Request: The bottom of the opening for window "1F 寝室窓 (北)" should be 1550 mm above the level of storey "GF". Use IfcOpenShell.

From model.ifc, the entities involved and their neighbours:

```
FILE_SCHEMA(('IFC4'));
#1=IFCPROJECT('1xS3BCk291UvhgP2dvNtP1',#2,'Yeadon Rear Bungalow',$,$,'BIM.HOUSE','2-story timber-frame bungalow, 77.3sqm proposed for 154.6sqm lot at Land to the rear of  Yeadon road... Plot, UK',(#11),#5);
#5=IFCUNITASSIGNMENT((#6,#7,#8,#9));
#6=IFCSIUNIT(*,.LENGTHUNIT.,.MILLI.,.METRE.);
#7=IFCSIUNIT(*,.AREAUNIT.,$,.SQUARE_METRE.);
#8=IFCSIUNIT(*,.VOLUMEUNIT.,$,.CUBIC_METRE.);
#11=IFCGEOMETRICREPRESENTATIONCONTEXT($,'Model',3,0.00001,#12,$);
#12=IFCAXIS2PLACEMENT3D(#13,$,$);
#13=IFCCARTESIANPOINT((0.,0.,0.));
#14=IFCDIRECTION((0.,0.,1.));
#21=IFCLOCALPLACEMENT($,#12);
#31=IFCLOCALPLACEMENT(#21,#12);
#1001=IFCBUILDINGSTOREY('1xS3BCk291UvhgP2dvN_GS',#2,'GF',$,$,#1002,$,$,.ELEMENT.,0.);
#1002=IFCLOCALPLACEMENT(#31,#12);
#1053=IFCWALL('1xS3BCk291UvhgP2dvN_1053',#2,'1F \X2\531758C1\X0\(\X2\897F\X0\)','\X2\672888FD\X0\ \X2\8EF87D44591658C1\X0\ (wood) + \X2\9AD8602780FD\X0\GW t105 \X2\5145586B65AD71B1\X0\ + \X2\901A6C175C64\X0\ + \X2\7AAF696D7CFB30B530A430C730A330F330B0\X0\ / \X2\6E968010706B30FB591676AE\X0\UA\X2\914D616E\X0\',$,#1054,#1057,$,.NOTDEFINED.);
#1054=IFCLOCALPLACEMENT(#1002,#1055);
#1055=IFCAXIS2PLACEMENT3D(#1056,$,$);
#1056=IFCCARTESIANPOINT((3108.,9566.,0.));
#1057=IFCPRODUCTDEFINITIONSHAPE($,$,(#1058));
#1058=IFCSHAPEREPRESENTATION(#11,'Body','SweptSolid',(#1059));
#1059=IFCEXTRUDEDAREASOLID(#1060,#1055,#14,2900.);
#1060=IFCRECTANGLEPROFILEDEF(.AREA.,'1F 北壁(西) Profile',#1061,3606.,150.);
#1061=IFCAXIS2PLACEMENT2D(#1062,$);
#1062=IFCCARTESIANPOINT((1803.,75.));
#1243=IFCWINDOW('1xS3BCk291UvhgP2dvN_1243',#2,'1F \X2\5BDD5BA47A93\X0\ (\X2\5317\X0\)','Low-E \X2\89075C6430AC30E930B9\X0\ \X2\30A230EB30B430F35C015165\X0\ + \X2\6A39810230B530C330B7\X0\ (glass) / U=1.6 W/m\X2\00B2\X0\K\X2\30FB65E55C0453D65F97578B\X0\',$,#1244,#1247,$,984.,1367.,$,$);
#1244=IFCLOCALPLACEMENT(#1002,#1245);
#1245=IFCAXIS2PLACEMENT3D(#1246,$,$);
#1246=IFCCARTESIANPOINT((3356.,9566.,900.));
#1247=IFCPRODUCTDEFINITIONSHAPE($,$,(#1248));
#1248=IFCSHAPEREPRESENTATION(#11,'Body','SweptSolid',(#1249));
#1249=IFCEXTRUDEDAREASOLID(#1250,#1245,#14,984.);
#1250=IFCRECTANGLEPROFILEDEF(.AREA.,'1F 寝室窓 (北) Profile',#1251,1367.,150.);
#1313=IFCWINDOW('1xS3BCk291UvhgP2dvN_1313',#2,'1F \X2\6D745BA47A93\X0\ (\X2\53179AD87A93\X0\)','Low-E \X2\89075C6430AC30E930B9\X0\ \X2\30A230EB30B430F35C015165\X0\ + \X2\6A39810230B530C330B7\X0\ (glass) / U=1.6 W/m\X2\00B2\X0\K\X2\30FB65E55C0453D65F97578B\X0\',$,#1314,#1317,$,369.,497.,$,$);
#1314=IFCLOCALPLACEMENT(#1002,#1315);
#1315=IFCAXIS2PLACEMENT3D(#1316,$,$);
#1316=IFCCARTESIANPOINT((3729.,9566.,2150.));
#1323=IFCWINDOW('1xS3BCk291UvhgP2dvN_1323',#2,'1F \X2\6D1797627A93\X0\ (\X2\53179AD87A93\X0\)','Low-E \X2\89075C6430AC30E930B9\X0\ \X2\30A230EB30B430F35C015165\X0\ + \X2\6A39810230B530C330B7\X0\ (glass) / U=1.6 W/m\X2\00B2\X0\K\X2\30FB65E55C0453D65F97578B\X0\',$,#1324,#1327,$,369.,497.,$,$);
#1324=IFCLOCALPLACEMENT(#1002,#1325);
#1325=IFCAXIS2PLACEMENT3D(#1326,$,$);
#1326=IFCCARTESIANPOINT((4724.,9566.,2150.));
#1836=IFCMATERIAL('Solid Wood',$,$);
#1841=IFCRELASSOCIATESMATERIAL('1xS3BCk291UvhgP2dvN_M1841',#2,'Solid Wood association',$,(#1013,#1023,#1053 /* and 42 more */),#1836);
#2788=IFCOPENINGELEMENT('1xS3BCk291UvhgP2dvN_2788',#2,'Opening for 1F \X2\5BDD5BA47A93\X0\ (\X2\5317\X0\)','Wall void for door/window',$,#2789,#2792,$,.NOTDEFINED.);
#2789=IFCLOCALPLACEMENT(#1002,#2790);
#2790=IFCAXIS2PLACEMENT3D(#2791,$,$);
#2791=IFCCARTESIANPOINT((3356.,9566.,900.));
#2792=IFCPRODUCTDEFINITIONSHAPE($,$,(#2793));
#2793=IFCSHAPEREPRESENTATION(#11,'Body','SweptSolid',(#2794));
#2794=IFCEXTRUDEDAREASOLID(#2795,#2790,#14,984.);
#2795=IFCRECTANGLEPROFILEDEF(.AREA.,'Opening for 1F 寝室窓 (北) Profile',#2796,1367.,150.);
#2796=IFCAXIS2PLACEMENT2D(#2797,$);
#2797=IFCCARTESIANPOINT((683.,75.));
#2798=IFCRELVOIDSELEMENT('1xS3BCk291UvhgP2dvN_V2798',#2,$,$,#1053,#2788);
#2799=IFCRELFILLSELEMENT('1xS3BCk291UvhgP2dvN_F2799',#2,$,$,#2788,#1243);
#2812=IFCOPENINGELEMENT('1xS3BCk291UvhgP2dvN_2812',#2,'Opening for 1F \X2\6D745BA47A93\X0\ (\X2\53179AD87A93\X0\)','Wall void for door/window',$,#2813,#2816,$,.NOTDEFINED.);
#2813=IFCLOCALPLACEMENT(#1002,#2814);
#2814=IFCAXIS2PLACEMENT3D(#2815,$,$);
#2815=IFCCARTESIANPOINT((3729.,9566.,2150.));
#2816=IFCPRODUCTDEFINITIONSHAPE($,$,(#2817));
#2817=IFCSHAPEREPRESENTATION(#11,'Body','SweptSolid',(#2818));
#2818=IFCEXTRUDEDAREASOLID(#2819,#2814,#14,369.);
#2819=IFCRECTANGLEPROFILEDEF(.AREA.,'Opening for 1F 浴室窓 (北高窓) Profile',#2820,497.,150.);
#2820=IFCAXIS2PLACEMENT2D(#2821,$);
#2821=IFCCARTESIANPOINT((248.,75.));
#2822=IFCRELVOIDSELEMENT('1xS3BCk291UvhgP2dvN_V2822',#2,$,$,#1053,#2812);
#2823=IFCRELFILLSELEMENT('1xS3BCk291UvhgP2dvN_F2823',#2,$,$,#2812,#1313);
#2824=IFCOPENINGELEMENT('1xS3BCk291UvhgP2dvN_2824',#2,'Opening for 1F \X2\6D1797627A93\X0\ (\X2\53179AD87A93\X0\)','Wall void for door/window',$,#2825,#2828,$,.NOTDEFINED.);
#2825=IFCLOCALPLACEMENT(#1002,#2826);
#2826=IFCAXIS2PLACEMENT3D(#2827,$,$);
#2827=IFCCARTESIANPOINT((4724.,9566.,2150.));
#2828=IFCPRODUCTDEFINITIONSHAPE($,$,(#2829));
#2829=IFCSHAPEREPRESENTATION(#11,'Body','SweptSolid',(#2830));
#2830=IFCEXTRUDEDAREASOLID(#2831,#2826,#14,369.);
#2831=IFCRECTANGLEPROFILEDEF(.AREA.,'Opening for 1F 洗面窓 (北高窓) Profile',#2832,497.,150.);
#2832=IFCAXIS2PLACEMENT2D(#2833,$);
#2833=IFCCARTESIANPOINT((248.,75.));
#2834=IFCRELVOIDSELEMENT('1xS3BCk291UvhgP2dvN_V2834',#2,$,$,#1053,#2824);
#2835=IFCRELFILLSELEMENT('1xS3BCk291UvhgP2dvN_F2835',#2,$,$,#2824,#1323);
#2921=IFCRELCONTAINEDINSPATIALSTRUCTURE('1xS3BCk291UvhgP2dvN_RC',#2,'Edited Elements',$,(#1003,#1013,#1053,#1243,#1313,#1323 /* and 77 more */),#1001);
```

```python
import numpy as np
import ifcopenshell
import ifcopenshell.api.geometry
import ifcopenshell.geom
import ifcopenshell.util.element
import ifcopenshell.util.placement
import ifcopenshell.util.shape
import ifcopenshell.util.unit

model = ifcopenshell.open("model.ifc")
unit_scale = ifcopenshell.util.unit.calculate_unit_scale(model)

window = model.by_guid("1xS3BCk291UvhgP2dvN_1243")
opening = window.FillsVoids[0].RelatingOpeningElement
storey = ifcopenshell.util.element.get_container(window, ifc_class="IfcBuildingStorey")
level = ifcopenshell.util.placement.get_local_placement(storey.ObjectPlacement)[2, 3]

# The opening's origin need not be at the sill, so measure its lowest point.
shape = ifcopenshell.geom.create_shape(ifcopenshell.geom.settings(), opening)
bottom = ifcopenshell.util.shape.get_shape_bottom_elevation(shape, shape.geometry) / unit_scale
dz = level + 1.55 / unit_scale - bottom

shift = np.array([0.0, 0.0, dz])
# The window is not placed relative to its opening, so move both.
for product in (opening, window):
    matrix = ifcopenshell.util.placement.get_local_placement(product.ObjectPlacement)
    matrix[:3, 3] += shift
    ifcopenshell.api.geometry.edit_object_placement(model, product=product, matrix=matrix, is_si=False)

print(f"moved by {dz * unit_scale:+.3f} m")

model.write("model_updated.ifc")
```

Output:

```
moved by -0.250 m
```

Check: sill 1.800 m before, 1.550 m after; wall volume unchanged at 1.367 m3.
